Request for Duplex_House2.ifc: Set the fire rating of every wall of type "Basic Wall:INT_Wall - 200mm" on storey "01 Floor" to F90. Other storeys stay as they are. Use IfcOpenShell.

First a look at what the model holds.

```python
import ifcopenshell
import ifcopenshell.util.element

model = ifcopenshell.open("Duplex_House2.ifc")
print(model.schema)
storey = next(s for s in model.by_type("IfcBuildingStorey") if s.Name == "01 Floor")
walls = [e for e in ifcopenshell.util.element.get_decomposition(storey) if e.is_a("IfcWall")]
seen = {}
for e in walls:
    element_type = ifcopenshell.util.element.get_type(e)
    key = (element_type.Name if element_type != e and element_type else None, ifcopenshell.util.element.get_pset(e, "Pset_WallCommon", "FireRating"))
    seen[key] = seen.get(key, 0) + 1
for (name, value), count in sorted(seen.items(), key=str):
    print(count, "x", name, "|", value)
```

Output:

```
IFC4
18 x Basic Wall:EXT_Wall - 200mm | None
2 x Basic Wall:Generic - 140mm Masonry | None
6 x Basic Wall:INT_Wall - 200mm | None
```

```python
import ifcopenshell
import ifcopenshell.api.pset
import ifcopenshell.util.element

model = ifcopenshell.open("Duplex_House2.ifc")

storey = next(s for s in model.by_type("IfcBuildingStorey") if s.Name == "01 Floor")
walls = [e for e in ifcopenshell.util.element.get_decomposition(storey) if e.is_a("IfcWall")]

count = 0
for e in walls:
    element_type = ifcopenshell.util.element.get_type(e)
    if element_type in (None, e) or element_type.Name != "Basic Wall:INT_Wall - 200mm":
        continue
    # add_pset returns the element's existing set when there is one.
    pset = ifcopenshell.api.pset.add_pset(model, product=e, name="Pset_WallCommon")
    ifcopenshell.api.pset.edit_pset(model, pset=pset, properties={"FireRating": "F90"})
    count += 1

print(count, "walls updated")

model.write("Duplex_House2_rev.ifc")
```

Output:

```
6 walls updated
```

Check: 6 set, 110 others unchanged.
